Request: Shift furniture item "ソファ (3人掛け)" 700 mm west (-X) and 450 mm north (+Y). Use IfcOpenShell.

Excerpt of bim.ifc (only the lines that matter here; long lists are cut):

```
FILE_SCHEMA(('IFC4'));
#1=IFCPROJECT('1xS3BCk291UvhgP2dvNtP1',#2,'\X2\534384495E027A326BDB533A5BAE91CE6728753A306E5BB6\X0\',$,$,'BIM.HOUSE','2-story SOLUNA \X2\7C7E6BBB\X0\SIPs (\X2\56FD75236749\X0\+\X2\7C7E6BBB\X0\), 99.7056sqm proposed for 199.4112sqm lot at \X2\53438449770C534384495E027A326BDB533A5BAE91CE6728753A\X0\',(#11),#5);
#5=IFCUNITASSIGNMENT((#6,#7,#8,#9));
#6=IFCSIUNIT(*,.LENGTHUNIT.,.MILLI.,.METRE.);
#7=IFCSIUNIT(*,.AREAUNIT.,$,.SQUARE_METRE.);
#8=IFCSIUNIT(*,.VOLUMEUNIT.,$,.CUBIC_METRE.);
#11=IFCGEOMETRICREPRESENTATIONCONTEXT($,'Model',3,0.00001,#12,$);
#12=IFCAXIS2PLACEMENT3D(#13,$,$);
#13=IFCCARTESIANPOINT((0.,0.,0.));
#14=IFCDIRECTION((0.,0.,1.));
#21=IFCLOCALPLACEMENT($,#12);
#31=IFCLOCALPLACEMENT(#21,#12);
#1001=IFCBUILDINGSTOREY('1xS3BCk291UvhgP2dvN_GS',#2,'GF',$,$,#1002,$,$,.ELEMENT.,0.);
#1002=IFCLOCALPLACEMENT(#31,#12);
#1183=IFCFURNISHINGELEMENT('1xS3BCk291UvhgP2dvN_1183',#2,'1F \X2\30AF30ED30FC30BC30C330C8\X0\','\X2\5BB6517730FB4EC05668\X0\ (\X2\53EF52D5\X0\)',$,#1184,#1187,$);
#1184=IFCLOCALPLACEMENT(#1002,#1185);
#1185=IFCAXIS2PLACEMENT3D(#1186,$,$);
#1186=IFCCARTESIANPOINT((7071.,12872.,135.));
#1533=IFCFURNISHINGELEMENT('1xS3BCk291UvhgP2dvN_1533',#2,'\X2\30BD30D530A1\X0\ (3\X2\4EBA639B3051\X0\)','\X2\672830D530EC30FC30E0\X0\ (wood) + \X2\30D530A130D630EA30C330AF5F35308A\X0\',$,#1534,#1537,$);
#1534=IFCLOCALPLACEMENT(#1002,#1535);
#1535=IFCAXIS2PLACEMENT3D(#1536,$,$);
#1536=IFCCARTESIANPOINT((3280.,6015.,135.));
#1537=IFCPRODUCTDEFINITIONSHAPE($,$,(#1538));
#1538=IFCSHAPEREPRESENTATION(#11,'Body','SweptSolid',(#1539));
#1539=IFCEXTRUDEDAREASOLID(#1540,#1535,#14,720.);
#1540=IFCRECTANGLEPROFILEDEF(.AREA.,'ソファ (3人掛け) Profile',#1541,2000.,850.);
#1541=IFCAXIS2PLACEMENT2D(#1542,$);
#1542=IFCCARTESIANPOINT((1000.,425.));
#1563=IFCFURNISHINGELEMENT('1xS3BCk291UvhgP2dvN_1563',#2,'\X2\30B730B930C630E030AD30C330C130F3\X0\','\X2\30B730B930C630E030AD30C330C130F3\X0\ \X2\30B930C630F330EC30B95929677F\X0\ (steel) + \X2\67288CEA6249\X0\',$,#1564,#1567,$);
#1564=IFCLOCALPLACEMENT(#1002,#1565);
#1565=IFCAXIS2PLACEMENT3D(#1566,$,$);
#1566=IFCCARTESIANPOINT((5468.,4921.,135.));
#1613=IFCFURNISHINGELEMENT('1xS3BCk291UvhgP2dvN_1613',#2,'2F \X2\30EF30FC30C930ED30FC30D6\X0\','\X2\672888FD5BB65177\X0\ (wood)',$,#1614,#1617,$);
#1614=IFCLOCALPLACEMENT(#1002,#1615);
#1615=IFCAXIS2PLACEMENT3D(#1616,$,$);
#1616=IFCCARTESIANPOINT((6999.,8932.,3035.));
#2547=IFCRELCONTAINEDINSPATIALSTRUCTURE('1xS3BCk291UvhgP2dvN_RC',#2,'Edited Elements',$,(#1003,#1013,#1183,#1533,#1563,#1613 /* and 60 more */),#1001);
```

```python
import ifcopenshell
import ifcopenshell.api.geometry
import ifcopenshell.util.placement
import ifcopenshell.util.unit

model = ifcopenshell.open("bim.ifc")
unit_scale = ifcopenshell.util.unit.calculate_unit_scale(model)

item = model.by_id(1533)
matrix = ifcopenshell.util.placement.get_local_placement(item.ObjectPlacement)
matrix[0, 3] -= 0.7 / unit_scale
matrix[1, 3] += 0.45 / unit_scale
ifcopenshell.api.geometry.edit_object_placement(model, product=item, matrix=matrix, is_si=False)

print(ifcopenshell.util.placement.get_local_placement(item.ObjectPlacement).round(3) + 0.0)

model.write("bim_edited.ifc")
```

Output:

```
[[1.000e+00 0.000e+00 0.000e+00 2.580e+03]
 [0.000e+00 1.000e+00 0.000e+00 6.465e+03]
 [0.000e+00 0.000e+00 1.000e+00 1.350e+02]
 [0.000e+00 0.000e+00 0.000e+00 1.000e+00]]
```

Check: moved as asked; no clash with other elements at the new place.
